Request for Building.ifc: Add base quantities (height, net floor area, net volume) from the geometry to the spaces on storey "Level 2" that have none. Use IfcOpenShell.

First a look at what the model holds.

```python
import ifcopenshell
import ifcopenshell.util.element
import ifcopenshell.util.unit

model = ifcopenshell.open("Building.ifc")
print(model.schema)
for unit_type in ("LENGTHUNIT", "AREAUNIT", "VOLUMEUNIT"):
    print(unit_type, ifcopenshell.util.unit.calculate_unit_scale(model, unit_type))
storey = next(s for s in model.by_type("IfcBuildingStorey") if s.Name == "Level 2")
spaces = [e for e in ifcopenshell.util.element.get_decomposition(storey) if e.is_a("IfcSpace")]
for e in sorted(spaces, key=lambda e: e.id()):
    print(e.id(), e.is_a(), e.Name, list(ifcopenshell.util.element.get_psets(e, qtos_only=True)), sep=" | ")
```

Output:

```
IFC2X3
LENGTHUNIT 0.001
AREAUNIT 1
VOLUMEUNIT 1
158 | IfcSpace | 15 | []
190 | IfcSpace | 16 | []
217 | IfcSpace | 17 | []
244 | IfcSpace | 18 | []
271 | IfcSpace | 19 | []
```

```python
import ifcopenshell
import ifcopenshell.api.pset
import ifcopenshell.geom
import ifcopenshell.util.element
import ifcopenshell.util.shape
import ifcopenshell.util.unit

model = ifcopenshell.open("Building.ifc")
unit_scale = ifcopenshell.util.unit.calculate_unit_scale(model)
area_scale = ifcopenshell.util.unit.calculate_unit_scale(model, "AREAUNIT")
volume_scale = ifcopenshell.util.unit.calculate_unit_scale(model, "VOLUMEUNIT")
settings = ifcopenshell.geom.settings()

storey = next(s for s in model.by_type("IfcBuildingStorey") if s.Name == "Level 2")
spaces = [e for e in ifcopenshell.util.element.get_decomposition(storey) if e.is_a("IfcSpace")]

for e in sorted(spaces, key=lambda e: e.id()):
    if ifcopenshell.util.element.get_psets(e, qtos_only=True, should_inherit=False):
        continue
    # Geometry comes back in metres, in the element's own axes.
    shape = ifcopenshell.geom.create_shape(settings, e)
    values = {
        "Height": ifcopenshell.util.shape.get_z(shape.geometry) / unit_scale,
        "NetFloorArea": ifcopenshell.util.shape.get_footprint_area(shape.geometry) / area_scale,
        "NetVolume": ifcopenshell.util.shape.get_volume(shape.geometry) / volume_scale,
    }
    qto = ifcopenshell.api.pset.add_qto(model, product=e, name="BaseQuantities")
    ifcopenshell.api.pset.edit_qto(model, qto=qto, properties=values)
    print(e.id(), {k: round(v, 3) for k, v in values.items()})

model.write("Building-out.ifc")
```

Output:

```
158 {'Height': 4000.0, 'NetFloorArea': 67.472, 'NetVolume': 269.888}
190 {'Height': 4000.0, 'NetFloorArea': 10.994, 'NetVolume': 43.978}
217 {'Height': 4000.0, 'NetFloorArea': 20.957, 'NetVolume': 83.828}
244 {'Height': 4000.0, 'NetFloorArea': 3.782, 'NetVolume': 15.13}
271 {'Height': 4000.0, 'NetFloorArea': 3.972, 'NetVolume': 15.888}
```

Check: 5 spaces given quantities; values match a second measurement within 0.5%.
